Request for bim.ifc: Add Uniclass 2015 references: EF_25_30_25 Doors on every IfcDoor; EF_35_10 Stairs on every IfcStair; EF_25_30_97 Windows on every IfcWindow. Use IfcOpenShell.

First a look at what the model holds.

```python
import ifcopenshell

model = ifcopenshell.open("bim.ifc")
print(model.schema)
print("classifications:", [c.Name for c in model.by_type("IfcClassification")])
for ifc_class in ("IfcDoor", "IfcRoof", "IfcStair", "IfcWall", "IfcWindow"):
    print(ifc_class, len(model.by_type(ifc_class)))
```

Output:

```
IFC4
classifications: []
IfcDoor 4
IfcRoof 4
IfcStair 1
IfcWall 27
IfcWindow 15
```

```python
import ifcopenshell
import ifcopenshell.api.classification

model = ifcopenshell.open("bim.ifc")

system = ifcopenshell.api.classification.add_classification(model, classification="Uniclass 2015")

codes = {
    "IfcDoor": ("EF_25_30_25", "Doors"),
    "IfcStair": ("EF_35_10", "Stairs"),
    "IfcWindow": ("EF_25_30_97", "Windows"),
}
for ifc_class, (code, name) in codes.items():
    products = model.by_type(ifc_class)
    ifcopenshell.api.classification.add_reference(
        model, products=products, classification=system, identification=code, name=name
    )
    print(code, len(products))

model.write("bim-out.ifc")
```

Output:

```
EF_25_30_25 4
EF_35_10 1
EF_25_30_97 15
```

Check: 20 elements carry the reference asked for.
